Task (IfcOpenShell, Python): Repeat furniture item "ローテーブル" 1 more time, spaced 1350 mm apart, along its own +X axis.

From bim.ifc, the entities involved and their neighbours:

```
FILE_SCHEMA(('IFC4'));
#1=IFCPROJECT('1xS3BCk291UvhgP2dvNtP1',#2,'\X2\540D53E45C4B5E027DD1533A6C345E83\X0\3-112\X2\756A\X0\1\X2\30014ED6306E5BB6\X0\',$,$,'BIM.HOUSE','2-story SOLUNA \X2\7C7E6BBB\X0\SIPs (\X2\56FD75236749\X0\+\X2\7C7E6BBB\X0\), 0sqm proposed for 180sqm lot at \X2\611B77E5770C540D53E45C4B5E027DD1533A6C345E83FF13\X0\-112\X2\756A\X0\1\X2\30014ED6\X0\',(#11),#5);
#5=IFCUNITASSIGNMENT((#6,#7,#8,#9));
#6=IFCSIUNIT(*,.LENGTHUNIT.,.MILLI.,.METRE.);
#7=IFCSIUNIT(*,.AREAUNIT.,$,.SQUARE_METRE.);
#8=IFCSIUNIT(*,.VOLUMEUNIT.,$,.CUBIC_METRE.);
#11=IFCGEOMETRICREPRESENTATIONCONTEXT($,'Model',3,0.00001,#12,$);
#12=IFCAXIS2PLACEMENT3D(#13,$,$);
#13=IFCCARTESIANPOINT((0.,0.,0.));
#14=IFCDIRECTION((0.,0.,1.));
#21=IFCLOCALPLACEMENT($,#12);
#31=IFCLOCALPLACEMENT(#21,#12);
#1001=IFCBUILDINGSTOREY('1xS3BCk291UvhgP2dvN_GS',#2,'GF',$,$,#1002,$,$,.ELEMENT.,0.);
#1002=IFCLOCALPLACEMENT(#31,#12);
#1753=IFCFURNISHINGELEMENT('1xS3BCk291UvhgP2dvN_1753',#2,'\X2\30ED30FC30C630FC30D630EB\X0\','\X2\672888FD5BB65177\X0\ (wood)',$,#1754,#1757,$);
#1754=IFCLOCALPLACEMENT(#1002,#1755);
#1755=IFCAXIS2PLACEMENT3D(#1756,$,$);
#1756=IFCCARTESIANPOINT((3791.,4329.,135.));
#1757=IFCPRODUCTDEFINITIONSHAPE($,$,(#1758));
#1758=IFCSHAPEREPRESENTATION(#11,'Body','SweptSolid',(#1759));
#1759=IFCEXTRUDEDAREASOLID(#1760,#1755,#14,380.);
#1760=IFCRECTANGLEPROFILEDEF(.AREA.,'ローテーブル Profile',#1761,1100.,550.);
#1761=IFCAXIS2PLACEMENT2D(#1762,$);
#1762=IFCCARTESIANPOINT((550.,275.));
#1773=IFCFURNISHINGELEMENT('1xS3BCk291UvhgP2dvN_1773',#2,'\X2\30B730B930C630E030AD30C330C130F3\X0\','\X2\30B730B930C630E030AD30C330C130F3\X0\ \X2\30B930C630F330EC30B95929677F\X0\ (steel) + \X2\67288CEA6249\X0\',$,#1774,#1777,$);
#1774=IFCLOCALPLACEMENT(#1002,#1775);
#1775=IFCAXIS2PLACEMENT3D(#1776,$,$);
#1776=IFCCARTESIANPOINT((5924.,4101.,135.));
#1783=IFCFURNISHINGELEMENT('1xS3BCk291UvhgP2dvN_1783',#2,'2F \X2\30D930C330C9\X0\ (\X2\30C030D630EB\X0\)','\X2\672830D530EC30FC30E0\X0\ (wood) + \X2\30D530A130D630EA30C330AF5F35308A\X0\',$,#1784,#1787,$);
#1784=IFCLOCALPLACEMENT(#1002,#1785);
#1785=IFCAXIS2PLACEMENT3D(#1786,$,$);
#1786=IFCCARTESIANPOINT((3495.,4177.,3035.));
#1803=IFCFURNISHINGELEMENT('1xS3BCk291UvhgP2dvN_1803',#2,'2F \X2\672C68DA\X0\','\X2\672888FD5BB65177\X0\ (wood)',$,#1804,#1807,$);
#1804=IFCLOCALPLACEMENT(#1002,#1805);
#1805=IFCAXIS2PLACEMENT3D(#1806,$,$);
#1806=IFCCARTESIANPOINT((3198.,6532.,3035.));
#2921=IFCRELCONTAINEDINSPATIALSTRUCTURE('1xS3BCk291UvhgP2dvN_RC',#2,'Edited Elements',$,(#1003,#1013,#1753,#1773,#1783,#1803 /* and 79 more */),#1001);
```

```python
import ifcopenshell
import ifcopenshell.api.geometry
import ifcopenshell.api.root
import ifcopenshell.util.element
import ifcopenshell.util.placement
import ifcopenshell.util.unit

model = ifcopenshell.open("bim.ifc")
unit_scale = ifcopenshell.util.unit.calculate_unit_scale(model)


def reuse_history(source, copy):
    """copy_class also copies each property set's owner history, people and application; keep the originals."""
    for rel in copy.IsDefinedBy:
        if rel.is_a("IfcRelDefinesByProperties") and (history := rel.RelatingPropertyDefinition.OwnerHistory):
            rel.RelatingPropertyDefinition.OwnerHistory = source.OwnerHistory
            ifcopenshell.util.element.remove_deep2(model, history)


source = model.by_guid("1xS3BCk291UvhgP2dvN_1753")
base = ifcopenshell.util.placement.get_local_placement(source.ObjectPlacement)
step = base[:3, 0] * 1.35 / unit_scale

for i in range(1, 2):
    copy = ifcopenshell.api.root.copy_class(model, product=source)
    copy.Representation = ifcopenshell.util.element.copy_deep(
        model, source.Representation, exclude=["IfcGeometricRepresentationContext", "IfcRepresentationMap"]
    )
    reuse_history(source, copy)
    matrix = base.copy()
    matrix[:3, 3] += i * step
    print("added at", matrix[:3, 3].round(3) + 0.0)
    ifcopenshell.api.geometry.edit_object_placement(model, product=copy, matrix=matrix, is_si=False)

model.write("bim_v2.ifc")
```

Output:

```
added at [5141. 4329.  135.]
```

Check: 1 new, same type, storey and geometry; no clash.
